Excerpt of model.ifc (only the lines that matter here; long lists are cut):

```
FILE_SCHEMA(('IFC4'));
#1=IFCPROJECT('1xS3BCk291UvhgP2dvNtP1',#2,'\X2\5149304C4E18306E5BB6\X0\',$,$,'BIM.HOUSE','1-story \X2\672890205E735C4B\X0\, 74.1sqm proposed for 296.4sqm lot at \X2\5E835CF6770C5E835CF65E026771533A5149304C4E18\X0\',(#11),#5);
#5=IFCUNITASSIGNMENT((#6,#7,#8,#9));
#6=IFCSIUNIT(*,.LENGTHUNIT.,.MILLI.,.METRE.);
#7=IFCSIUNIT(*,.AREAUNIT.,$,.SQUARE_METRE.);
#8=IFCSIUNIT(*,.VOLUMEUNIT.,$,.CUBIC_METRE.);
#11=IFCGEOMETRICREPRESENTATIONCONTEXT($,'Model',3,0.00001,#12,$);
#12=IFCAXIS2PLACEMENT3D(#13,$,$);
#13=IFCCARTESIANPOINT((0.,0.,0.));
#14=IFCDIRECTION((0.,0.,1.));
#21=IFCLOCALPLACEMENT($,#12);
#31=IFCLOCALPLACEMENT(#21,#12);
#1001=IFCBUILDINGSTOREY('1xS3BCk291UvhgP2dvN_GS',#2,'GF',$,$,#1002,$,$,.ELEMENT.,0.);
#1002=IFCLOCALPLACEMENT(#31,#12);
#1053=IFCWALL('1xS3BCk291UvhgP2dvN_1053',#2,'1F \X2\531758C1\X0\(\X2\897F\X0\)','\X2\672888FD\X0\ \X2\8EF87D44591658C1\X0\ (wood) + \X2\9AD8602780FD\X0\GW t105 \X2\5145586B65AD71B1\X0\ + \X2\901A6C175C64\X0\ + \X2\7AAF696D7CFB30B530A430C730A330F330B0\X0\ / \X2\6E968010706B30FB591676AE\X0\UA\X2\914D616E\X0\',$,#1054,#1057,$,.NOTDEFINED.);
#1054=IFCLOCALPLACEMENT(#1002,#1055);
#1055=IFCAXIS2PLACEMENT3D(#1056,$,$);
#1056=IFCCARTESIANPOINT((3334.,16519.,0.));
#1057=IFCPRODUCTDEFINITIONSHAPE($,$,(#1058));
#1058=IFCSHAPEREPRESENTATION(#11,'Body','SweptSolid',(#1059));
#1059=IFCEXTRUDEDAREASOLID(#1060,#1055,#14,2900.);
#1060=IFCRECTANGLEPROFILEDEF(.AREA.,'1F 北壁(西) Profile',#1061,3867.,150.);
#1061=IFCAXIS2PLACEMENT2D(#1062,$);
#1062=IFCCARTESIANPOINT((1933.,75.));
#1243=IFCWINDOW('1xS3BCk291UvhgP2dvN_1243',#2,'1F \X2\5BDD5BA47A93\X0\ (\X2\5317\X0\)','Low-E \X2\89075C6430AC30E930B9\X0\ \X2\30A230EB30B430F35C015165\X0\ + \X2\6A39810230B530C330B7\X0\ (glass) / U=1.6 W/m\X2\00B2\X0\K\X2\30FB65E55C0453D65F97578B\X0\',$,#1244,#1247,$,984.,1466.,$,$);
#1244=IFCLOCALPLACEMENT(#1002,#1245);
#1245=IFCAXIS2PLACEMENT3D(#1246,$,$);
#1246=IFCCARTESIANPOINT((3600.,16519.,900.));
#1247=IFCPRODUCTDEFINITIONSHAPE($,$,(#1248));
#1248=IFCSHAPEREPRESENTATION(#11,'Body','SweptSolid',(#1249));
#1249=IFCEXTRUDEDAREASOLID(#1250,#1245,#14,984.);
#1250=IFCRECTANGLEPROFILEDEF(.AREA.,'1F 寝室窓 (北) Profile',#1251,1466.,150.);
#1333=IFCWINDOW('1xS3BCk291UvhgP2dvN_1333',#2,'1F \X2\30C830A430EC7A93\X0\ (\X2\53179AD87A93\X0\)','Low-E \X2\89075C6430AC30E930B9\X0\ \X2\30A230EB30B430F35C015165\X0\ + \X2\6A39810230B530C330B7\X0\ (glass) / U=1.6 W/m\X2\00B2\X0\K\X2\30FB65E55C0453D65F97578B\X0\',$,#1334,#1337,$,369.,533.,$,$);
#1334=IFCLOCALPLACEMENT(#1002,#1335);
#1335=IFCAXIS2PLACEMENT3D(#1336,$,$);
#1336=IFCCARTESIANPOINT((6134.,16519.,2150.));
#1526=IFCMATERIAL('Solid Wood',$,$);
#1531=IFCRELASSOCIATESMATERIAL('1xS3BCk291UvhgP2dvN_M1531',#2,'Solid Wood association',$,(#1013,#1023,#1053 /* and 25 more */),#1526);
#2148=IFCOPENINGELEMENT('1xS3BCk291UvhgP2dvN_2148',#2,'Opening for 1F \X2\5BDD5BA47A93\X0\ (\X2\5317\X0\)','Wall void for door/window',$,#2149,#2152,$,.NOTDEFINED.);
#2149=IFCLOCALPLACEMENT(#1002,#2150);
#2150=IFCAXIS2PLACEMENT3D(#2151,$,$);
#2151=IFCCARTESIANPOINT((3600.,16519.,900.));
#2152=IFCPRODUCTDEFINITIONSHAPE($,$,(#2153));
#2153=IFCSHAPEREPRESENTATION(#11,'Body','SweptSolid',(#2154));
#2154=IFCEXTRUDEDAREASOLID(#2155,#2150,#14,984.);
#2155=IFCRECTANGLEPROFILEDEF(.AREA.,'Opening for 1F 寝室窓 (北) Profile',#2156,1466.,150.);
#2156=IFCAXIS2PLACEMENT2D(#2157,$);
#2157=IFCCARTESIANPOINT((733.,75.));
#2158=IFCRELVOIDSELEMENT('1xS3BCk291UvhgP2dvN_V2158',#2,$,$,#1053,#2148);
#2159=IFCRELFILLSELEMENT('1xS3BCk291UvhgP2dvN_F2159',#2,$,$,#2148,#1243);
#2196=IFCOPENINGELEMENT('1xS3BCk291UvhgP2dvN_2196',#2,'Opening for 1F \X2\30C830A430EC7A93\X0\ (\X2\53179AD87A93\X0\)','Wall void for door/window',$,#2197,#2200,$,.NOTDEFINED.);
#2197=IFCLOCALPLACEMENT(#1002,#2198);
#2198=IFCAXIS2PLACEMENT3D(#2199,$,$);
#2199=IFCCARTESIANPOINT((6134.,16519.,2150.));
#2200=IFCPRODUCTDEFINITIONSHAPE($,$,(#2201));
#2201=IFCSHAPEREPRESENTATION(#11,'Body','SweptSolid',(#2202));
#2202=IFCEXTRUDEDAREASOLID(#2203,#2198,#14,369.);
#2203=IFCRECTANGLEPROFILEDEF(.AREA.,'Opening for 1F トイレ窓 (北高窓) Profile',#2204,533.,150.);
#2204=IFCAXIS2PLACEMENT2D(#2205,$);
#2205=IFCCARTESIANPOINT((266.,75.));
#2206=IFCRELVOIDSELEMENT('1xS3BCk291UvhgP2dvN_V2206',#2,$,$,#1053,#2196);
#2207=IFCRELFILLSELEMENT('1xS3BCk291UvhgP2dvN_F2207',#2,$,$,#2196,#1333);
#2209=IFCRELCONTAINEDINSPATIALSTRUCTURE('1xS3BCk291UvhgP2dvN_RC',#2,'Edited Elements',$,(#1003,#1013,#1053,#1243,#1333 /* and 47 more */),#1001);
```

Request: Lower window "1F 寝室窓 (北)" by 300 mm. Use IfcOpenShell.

```python
import numpy as np
import ifcopenshell
import ifcopenshell.api.geometry
import ifcopenshell.util.placement
import ifcopenshell.util.unit

model = ifcopenshell.open("model.ifc")
unit_scale = ifcopenshell.util.unit.calculate_unit_scale(model)

window = model.by_id(1243)
opening = window.FillsVoids[0].RelatingOpeningElement
dz = -0.3 / unit_scale

shift = np.array([0.0, 0.0, dz])
# The window is not placed relative to its opening, so move both.
for product in (opening, window):
    matrix = ifcopenshell.util.placement.get_local_placement(product.ObjectPlacement)
    matrix[:3, 3] += shift
    ifcopenshell.api.geometry.edit_object_placement(model, product=product, matrix=matrix, is_si=False)

print(f"moved by {dz * unit_scale:+.3f} m")

model.write("model_updated.ifc")
```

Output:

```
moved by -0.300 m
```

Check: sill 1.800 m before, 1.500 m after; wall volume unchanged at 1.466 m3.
